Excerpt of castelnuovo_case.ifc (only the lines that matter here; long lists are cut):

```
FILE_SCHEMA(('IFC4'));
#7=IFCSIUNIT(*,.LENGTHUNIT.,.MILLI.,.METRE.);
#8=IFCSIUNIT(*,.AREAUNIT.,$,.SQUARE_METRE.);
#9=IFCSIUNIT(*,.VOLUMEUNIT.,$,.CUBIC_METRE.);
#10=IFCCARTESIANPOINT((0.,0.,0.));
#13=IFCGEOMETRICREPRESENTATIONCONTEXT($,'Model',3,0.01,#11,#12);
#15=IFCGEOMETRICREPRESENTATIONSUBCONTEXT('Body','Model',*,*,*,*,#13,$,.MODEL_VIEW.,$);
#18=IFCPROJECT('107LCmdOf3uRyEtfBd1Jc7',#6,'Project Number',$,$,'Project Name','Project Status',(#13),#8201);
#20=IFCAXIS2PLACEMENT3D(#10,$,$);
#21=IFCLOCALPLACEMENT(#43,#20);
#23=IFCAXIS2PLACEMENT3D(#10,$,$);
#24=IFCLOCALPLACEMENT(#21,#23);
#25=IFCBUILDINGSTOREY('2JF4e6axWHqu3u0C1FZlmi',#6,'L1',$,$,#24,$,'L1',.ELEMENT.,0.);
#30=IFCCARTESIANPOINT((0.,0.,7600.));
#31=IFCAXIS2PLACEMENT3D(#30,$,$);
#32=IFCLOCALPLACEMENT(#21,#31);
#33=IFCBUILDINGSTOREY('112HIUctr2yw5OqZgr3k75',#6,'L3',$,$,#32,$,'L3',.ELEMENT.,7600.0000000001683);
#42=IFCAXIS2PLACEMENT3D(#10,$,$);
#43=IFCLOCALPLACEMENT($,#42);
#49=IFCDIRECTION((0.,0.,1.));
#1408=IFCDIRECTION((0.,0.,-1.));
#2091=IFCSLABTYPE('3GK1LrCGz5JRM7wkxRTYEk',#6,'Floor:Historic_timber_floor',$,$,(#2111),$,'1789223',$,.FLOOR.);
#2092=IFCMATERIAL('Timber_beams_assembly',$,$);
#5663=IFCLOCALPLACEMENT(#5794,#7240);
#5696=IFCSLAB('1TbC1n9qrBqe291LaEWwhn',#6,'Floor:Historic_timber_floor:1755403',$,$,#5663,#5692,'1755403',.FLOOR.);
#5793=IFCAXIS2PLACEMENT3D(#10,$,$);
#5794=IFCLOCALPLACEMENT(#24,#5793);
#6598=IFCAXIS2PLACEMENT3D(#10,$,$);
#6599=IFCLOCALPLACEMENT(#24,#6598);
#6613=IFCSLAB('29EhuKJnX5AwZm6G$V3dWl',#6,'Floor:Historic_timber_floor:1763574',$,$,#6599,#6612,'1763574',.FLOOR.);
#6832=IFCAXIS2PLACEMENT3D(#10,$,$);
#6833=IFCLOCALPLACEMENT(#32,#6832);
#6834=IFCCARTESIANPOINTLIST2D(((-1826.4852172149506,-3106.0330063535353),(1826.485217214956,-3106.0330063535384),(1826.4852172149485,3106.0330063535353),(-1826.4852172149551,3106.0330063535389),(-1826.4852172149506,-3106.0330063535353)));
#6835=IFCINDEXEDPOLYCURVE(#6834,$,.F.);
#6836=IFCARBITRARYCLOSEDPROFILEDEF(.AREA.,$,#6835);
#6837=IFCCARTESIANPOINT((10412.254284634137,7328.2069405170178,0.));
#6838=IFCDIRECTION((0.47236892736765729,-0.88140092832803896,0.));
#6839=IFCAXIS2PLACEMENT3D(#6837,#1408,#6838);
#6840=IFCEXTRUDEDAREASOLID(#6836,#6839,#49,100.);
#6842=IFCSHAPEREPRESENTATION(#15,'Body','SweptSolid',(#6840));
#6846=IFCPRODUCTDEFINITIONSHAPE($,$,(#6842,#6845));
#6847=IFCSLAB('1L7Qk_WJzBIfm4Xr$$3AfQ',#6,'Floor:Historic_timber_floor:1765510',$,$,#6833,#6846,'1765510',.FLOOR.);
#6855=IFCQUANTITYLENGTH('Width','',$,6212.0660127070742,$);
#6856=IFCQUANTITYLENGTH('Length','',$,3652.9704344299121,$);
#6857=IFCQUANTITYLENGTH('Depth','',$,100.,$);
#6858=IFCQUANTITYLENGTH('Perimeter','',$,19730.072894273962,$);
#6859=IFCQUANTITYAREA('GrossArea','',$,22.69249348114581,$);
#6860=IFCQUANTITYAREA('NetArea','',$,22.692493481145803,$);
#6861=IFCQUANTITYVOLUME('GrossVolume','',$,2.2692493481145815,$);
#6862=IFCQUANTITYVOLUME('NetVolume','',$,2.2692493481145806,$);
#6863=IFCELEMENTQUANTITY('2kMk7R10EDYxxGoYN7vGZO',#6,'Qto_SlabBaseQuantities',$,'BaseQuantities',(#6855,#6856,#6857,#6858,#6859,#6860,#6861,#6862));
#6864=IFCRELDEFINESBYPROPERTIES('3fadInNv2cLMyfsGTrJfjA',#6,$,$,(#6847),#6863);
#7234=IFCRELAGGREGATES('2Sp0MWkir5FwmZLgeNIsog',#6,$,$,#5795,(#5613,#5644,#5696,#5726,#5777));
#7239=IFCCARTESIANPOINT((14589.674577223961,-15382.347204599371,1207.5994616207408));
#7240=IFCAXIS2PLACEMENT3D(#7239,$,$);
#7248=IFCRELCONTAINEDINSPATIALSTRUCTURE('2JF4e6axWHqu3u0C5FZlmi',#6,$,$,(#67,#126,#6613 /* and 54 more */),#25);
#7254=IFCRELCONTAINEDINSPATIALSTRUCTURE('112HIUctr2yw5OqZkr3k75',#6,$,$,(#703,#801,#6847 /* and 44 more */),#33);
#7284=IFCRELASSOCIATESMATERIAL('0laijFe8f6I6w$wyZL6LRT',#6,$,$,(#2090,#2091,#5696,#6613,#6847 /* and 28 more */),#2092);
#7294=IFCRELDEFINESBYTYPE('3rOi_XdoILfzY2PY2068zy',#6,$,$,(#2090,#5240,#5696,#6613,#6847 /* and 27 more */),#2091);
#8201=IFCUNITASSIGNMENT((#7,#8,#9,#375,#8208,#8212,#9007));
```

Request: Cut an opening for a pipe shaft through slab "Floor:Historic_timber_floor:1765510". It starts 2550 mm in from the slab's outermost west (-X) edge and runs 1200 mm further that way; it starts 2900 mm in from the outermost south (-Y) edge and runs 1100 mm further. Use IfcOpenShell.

```python
import numpy as np
import ifcopenshell
import ifcopenshell.api.feature
import ifcopenshell.api.geometry
import ifcopenshell.api.pset
import ifcopenshell.api.root
import ifcopenshell.geom
import ifcopenshell.util.element
import ifcopenshell.util.placement
import ifcopenshell.util.representation
import ifcopenshell.util.shape
import ifcopenshell.util.unit

model = ifcopenshell.open("castelnuovo_case.ifc")
unit_scale = ifcopenshell.util.unit.calculate_unit_scale(model)
area_scale = ifcopenshell.util.unit.calculate_unit_scale(model, "AREAUNIT")
volume_scale = ifcopenshell.util.unit.calculate_unit_scale(model, "VOLUMEUNIT")
settings = ifcopenshell.geom.settings()


def volume(element):
    """Net volume in cubic metres, openings subtracted."""
    shape = ifcopenshell.geom.create_shape(settings, element)
    return ifcopenshell.util.shape.get_volume(shape.geometry)


slab = model.by_guid("1L7Qk_WJzBIfm4Xr$$3AfQ")
before = volume(slab)

# Extent in the slab's own axes, in metres. The edges named are its -X and -Y sides.
slab_shape = ifcopenshell.geom.create_shape(settings, slab)
vertices = ifcopenshell.util.shape.get_vertices(slab_shape.geometry)
x_min, y_min, bottom = vertices.min(axis=0)
top = vertices[:, 2].max()

opening = ifcopenshell.api.root.create_entity(model, ifc_class="IfcOpeningElement", name="Pipe shaft opening", predefined_type="OPENING")
context = ifcopenshell.util.representation.get_context(model, "Model", "Body", "MODEL_VIEW")
width, depth = 1.2, 1.1
outline = [(0.0, 0.0), (width, 0.0), (width, depth), (0.0, depth), (0.0, 0.0)]
# Overshoot both faces by 50 mm so the cut is clean.
shape = ifcopenshell.api.geometry.add_slab_representation(
    model, context=context, depth=top - bottom + 0.1, polyline=outline
)
ifcopenshell.api.geometry.assign_representation(model, product=opening, representation=shape)

matrix = ifcopenshell.util.placement.get_local_placement(slab.ObjectPlacement)
matrix[:, 3] = matrix @ np.append(np.array([x_min + 2.55, y_min + 2.9, bottom - 0.05]) / unit_scale, 1.0)
ifcopenshell.api.geometry.edit_object_placement(model, product=opening, matrix=matrix, is_si=False)
ifcopenshell.api.feature.add_feature(model, feature=opening, element=slab)

after = volume(slab)

# Update the slab's stored quantities.
qto = model.by_id(ifcopenshell.util.element.get_pset(slab, "Qto_SlabBaseQuantities", should_inherit=False)["id"])
ifcopenshell.api.pset.edit_qto(model, qto=qto, properties={
    "NetArea": after / (top - bottom) / area_scale,
    "NetVolume": after / volume_scale,
})

print(f"slab volume {before:.3f} -> {after:.3f} m3")

model.write("castelnuovo_case-out.ifc")
```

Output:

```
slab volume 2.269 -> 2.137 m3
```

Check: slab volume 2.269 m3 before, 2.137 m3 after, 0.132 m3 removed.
